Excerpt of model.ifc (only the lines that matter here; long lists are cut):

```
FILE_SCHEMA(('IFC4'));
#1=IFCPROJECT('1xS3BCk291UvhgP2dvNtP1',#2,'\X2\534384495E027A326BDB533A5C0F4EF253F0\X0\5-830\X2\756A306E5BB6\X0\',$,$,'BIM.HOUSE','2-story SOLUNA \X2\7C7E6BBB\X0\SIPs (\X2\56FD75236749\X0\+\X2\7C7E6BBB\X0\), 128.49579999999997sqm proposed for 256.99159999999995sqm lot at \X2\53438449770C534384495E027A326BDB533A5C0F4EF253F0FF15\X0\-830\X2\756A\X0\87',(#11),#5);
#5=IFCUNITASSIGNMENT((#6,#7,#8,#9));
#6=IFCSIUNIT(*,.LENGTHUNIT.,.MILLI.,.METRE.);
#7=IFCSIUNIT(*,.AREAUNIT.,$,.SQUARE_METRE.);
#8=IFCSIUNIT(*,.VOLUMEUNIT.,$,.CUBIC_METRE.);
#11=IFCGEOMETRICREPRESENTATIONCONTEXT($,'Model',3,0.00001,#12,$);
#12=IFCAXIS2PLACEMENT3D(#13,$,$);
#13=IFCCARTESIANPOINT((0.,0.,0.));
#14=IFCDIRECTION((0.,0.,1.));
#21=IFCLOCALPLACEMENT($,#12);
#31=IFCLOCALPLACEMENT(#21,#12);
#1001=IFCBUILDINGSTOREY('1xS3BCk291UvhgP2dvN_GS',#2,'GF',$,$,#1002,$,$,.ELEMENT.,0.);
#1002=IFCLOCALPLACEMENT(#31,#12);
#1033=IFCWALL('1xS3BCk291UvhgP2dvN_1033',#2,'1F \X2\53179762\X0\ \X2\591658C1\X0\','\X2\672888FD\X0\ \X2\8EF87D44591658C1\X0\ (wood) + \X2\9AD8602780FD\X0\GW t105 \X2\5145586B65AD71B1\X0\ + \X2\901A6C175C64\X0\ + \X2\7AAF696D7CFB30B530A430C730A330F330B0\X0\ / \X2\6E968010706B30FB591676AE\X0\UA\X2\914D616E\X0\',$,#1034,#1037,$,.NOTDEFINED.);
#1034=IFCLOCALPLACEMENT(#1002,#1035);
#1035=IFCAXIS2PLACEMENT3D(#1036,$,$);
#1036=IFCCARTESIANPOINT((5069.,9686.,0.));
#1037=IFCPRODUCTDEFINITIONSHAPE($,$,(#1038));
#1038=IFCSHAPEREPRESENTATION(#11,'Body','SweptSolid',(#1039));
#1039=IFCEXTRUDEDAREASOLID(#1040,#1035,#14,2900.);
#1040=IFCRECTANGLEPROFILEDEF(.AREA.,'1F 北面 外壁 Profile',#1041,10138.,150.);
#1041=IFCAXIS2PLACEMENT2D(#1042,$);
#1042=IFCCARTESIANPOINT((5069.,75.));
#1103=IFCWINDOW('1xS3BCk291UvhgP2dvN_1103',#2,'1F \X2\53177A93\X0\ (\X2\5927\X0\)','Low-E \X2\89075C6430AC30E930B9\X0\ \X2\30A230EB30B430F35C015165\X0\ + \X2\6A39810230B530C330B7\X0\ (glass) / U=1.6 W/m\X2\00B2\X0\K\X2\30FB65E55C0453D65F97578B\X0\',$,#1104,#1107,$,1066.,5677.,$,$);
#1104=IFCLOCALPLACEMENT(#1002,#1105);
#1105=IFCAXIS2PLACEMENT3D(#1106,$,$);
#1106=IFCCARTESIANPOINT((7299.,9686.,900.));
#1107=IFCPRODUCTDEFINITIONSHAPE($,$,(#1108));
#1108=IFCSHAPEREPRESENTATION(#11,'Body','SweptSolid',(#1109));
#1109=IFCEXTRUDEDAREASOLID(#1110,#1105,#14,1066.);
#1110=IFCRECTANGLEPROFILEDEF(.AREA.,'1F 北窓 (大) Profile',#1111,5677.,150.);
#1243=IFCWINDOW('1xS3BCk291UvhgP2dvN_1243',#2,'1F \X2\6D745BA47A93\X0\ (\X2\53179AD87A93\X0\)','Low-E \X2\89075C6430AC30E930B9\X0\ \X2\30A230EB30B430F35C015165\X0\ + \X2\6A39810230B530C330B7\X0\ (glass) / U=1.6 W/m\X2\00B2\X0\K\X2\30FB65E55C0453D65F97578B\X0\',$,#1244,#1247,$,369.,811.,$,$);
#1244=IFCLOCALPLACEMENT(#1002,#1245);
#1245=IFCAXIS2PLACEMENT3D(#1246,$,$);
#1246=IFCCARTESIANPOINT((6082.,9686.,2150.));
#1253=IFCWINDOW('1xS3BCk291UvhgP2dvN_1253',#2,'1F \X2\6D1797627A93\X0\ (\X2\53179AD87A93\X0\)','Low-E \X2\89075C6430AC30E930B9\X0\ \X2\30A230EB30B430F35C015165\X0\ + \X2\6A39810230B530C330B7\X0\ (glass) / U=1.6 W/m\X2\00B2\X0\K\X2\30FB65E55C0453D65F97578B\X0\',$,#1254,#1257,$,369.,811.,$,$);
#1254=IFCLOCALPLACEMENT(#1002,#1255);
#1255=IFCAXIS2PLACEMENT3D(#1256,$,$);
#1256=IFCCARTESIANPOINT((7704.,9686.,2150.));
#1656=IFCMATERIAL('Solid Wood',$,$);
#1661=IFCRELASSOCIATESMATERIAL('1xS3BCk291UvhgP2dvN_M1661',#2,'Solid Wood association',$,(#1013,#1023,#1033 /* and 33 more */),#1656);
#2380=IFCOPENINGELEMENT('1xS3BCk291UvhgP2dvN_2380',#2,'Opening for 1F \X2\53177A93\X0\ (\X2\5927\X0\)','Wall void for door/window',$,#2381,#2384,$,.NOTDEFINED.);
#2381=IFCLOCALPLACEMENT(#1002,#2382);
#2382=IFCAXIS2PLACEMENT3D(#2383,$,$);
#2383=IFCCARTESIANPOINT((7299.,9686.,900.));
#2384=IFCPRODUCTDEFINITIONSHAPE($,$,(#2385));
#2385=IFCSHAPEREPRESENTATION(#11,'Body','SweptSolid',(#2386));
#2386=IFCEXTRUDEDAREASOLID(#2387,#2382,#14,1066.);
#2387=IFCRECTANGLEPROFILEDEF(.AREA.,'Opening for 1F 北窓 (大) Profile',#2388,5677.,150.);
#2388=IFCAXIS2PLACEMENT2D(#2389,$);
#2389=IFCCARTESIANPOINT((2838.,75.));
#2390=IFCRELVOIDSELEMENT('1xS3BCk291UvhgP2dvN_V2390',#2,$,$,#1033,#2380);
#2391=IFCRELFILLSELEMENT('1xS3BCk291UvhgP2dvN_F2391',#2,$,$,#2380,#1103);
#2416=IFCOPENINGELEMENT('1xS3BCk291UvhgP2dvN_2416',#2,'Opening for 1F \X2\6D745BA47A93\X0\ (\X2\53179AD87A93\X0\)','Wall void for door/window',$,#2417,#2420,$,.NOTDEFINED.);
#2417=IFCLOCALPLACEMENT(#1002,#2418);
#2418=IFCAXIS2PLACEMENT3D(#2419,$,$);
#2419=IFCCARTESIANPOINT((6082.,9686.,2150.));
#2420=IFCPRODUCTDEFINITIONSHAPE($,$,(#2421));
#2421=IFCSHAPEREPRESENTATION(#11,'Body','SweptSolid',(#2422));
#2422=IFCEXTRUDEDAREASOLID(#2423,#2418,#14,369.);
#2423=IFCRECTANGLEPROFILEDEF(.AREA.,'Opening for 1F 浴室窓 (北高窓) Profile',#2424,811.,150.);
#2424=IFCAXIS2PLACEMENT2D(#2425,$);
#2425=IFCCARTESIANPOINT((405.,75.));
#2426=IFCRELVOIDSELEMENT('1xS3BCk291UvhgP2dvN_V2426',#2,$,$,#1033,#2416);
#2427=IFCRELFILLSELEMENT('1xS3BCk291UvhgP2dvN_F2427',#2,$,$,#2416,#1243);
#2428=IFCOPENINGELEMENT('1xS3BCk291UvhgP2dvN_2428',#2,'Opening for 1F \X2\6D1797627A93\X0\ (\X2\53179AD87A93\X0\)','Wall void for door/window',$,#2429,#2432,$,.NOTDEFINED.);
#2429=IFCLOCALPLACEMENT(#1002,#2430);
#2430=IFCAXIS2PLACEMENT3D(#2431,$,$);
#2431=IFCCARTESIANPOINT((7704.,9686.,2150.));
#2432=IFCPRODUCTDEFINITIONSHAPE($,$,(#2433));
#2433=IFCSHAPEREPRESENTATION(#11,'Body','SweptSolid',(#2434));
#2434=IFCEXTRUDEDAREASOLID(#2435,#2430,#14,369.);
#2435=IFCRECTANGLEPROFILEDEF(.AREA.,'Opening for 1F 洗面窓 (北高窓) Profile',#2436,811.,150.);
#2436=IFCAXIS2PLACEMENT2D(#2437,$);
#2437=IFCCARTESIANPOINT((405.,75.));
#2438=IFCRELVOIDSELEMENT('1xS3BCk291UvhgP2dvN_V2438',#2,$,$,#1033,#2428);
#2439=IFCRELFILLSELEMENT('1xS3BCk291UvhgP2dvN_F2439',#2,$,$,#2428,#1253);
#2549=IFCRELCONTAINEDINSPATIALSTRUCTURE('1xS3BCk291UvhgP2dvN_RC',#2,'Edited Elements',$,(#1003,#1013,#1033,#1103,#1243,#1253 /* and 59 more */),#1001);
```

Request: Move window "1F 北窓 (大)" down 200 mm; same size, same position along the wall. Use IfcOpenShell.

```python
import numpy as np
import ifcopenshell
import ifcopenshell.api.geometry
import ifcopenshell.util.placement
import ifcopenshell.util.unit

model = ifcopenshell.open("model.ifc")
unit_scale = ifcopenshell.util.unit.calculate_unit_scale(model)

window = model.by_guid("1xS3BCk291UvhgP2dvN_1103")
opening = window.FillsVoids[0].RelatingOpeningElement
dz = -200.0

shift = np.array([0.0, 0.0, dz])
# The window is not placed relative to its opening, so move both.
for product in (opening, window):
    matrix = ifcopenshell.util.placement.get_local_placement(product.ObjectPlacement)
    matrix[:3, 3] += shift
    ifcopenshell.api.geometry.edit_object_placement(model, product=product, matrix=matrix, is_si=False)

print(f"moved by {dz * unit_scale:+.3f} m")

model.write("model_edited.ifc")
```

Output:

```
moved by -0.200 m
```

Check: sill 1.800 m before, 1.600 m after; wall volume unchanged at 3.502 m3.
